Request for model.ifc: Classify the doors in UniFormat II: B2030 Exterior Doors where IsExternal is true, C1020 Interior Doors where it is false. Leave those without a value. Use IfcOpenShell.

First a look at what the model holds.

```python
import ifcopenshell
import ifcopenshell.util.element

model = ifcopenshell.open("model.ifc")
print(model.schema)
print("classifications:", [c.Name for c in model.by_type("IfcClassification")])
values = [ifcopenshell.util.element.get_pset(e, "Pset_DoorCommon", "IsExternal") for e in model.by_type("IfcDoor")]
for value in (True, False, None):
    print("IsExternal", value, values.count(value))
```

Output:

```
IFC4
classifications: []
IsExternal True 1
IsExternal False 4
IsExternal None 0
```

```python
import ifcopenshell
import ifcopenshell.api.classification
import ifcopenshell.util.element

model = ifcopenshell.open("model.ifc")

system = ifcopenshell.api.classification.add_classification(model, classification="UniFormat II")

doors = model.by_type("IfcDoor")
external = {e: ifcopenshell.util.element.get_pset(e, "Pset_DoorCommon", "IsExternal") for e in doors}
for flag, code, name in ((True, "B2030", "Exterior Doors"), (False, "C1020", "Interior Doors")):
    products = [e for e in doors if external[e] is flag]
    ifcopenshell.api.classification.add_reference(
        model, products=products, classification=system, identification=code, name=name
    )
    print(code, len(products))

model.write("model_rev.ifc")
```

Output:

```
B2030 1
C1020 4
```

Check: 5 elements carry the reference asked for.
